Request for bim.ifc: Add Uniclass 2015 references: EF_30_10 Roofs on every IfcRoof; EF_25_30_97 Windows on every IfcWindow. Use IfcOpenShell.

First a look at what the model holds.

```python
import ifcopenshell

model = ifcopenshell.open("bim.ifc")
print(model.schema)
print("classifications:", [c.Name for c in model.by_type("IfcClassification")])
for ifc_class in ("IfcDoor", "IfcRoof", "IfcStair", "IfcWall", "IfcWindow"):
    print(ifc_class, len(model.by_type(ifc_class)))
```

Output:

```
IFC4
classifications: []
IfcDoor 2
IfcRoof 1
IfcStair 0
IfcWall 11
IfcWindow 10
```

```python
import ifcopenshell
import ifcopenshell.api.classification

model = ifcopenshell.open("bim.ifc")

system = ifcopenshell.api.classification.add_classification(model, classification="Uniclass 2015")

codes = {
    "IfcRoof": ("EF_30_10", "Roofs"),
    "IfcWindow": ("EF_25_30_97", "Windows"),
}
for ifc_class, (code, name) in codes.items():
    products = model.by_type(ifc_class)
    ifcopenshell.api.classification.add_reference(
        model, products=products, classification=system, identification=code, name=name
    )
    print(code, len(products))

model.write("bim_rev.ifc")
```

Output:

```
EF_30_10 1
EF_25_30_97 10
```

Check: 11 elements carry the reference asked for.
